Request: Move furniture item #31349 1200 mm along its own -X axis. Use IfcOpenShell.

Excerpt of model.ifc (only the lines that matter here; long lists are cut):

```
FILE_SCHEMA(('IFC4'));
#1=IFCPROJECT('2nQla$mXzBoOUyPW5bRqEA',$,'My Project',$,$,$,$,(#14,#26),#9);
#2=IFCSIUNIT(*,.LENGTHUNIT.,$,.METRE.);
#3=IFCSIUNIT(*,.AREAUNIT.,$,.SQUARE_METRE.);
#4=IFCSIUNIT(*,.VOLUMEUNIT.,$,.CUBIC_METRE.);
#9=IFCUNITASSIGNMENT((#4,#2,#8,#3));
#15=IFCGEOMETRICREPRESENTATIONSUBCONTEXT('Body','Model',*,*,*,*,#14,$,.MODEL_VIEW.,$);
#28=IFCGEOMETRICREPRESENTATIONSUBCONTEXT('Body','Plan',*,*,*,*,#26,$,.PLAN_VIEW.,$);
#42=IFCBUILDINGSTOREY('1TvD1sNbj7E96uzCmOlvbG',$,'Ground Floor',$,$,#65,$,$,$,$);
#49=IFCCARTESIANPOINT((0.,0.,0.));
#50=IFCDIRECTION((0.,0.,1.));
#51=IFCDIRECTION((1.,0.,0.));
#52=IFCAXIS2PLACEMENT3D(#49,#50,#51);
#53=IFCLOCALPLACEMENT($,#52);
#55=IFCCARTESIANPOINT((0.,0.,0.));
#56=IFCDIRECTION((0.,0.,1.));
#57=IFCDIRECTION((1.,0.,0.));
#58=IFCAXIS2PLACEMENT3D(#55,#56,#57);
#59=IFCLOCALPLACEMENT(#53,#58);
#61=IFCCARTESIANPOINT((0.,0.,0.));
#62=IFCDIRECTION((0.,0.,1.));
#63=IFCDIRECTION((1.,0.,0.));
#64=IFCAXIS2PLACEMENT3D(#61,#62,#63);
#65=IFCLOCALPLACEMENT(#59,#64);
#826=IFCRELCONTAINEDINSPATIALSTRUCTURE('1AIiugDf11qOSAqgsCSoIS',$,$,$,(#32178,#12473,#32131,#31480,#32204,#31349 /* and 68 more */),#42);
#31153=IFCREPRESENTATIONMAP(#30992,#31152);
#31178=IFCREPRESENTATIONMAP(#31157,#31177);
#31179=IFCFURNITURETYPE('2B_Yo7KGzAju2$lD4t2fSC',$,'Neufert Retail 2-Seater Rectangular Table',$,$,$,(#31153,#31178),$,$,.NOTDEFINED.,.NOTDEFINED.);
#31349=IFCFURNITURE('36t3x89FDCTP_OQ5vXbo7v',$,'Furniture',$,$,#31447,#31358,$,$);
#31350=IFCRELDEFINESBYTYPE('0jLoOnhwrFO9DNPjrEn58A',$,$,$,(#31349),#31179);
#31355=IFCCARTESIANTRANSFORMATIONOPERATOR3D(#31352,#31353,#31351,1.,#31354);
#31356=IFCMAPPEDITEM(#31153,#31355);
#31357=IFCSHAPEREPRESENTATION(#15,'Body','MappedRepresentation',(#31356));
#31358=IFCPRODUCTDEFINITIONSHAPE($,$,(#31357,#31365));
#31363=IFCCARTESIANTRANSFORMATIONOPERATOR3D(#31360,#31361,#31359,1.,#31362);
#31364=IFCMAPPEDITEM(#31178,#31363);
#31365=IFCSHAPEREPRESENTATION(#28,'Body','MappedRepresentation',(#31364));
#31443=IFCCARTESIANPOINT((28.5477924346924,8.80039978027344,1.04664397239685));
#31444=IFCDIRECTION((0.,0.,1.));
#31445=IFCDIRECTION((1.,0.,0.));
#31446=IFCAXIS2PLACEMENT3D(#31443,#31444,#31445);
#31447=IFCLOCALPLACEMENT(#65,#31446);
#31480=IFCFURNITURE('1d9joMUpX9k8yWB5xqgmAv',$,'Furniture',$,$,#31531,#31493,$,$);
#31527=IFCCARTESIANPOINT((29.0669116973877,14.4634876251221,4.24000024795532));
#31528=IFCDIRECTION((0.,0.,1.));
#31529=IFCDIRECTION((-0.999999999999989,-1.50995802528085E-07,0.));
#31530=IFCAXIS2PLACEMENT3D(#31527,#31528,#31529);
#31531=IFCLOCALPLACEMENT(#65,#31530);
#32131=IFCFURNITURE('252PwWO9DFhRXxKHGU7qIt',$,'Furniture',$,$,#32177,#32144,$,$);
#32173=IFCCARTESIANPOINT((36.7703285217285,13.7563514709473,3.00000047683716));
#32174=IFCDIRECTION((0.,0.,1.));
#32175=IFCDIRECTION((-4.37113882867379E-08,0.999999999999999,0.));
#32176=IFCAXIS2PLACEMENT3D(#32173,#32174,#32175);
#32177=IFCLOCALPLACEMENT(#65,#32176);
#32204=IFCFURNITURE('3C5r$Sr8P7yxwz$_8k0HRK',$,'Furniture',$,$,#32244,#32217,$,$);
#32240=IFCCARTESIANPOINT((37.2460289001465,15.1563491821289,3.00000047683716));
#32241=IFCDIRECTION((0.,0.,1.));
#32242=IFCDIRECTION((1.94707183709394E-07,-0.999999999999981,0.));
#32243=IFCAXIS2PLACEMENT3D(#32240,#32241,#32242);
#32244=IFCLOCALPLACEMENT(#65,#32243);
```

```python
import ifcopenshell
import ifcopenshell.api.geometry
import ifcopenshell.util.placement

model = ifcopenshell.open("model.ifc")

item = model.by_guid("36t3x89FDCTP_OQ5vXbo7v")
matrix = ifcopenshell.util.placement.get_local_placement(item.ObjectPlacement)
matrix[:3, 3] -= matrix[:3, 0] * 1.2
ifcopenshell.api.geometry.edit_object_placement(model, product=item, matrix=matrix, is_si=False)

print(ifcopenshell.util.placement.get_local_placement(item.ObjectPlacement).round(3) + 0.0)

model.write("model-out.ifc")
```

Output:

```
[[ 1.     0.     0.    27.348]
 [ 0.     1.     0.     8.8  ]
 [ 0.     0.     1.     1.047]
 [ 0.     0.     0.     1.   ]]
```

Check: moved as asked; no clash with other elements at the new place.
